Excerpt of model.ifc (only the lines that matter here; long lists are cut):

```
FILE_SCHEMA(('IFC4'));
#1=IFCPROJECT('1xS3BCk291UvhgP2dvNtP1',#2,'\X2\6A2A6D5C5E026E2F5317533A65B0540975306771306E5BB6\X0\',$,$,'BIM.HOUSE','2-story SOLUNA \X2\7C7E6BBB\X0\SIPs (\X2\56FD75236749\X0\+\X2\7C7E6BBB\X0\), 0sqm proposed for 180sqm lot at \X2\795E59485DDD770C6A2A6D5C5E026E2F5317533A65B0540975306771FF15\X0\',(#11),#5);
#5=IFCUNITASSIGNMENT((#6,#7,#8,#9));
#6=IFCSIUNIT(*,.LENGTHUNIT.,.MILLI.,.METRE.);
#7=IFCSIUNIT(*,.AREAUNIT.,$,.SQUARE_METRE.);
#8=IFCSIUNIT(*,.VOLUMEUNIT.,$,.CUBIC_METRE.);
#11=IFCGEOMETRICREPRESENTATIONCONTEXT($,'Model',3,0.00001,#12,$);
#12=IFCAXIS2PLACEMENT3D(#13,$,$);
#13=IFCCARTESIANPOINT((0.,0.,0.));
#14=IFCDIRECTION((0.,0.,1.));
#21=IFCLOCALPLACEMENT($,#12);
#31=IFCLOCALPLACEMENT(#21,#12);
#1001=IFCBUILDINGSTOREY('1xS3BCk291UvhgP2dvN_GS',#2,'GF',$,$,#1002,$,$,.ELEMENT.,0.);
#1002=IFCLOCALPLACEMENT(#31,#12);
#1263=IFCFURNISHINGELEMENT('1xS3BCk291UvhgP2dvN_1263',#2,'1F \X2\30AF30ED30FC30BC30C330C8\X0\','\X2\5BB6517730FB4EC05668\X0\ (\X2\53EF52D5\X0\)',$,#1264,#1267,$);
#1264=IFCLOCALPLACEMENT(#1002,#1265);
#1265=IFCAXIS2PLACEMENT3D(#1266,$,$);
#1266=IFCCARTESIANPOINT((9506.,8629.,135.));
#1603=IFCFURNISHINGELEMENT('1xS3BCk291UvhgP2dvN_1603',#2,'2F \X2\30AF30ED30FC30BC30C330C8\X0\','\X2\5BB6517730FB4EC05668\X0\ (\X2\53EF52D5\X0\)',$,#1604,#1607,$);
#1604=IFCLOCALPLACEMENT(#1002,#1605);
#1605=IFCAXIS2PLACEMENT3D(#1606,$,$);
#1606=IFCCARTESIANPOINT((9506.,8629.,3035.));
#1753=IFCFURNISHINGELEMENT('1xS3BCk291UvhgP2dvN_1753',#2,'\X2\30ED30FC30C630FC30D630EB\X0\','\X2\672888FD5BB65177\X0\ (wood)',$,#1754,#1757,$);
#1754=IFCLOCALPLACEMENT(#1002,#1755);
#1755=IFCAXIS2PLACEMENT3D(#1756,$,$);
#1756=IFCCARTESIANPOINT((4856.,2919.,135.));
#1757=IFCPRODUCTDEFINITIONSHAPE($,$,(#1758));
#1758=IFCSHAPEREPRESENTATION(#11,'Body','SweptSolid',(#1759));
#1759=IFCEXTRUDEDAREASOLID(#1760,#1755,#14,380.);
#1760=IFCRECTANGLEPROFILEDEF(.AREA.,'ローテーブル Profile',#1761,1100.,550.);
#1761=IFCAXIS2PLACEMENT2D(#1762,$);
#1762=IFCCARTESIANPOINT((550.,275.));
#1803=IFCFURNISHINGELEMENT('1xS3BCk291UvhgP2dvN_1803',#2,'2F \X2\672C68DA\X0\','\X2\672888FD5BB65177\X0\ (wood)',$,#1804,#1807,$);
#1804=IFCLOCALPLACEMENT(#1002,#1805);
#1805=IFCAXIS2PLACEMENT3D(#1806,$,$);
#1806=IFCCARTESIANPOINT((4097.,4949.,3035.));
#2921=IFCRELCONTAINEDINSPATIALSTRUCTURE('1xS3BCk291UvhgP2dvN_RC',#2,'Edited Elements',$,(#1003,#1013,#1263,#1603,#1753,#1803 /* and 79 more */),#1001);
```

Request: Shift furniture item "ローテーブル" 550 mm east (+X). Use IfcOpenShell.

```python
import ifcopenshell
import ifcopenshell.api.geometry
import ifcopenshell.util.placement

model = ifcopenshell.open("model.ifc")

item = model.by_id(1753)
matrix = ifcopenshell.util.placement.get_local_placement(item.ObjectPlacement)
matrix[0, 3] += 550.0
ifcopenshell.api.geometry.edit_object_placement(model, product=item, matrix=matrix, is_si=False)

print(ifcopenshell.util.placement.get_local_placement(item.ObjectPlacement).round(3) + 0.0)

model.write("model-out.ifc")
```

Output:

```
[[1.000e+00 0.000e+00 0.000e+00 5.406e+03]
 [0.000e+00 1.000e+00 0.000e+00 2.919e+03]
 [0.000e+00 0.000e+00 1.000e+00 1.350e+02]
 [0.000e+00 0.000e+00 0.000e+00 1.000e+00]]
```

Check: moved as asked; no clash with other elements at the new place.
